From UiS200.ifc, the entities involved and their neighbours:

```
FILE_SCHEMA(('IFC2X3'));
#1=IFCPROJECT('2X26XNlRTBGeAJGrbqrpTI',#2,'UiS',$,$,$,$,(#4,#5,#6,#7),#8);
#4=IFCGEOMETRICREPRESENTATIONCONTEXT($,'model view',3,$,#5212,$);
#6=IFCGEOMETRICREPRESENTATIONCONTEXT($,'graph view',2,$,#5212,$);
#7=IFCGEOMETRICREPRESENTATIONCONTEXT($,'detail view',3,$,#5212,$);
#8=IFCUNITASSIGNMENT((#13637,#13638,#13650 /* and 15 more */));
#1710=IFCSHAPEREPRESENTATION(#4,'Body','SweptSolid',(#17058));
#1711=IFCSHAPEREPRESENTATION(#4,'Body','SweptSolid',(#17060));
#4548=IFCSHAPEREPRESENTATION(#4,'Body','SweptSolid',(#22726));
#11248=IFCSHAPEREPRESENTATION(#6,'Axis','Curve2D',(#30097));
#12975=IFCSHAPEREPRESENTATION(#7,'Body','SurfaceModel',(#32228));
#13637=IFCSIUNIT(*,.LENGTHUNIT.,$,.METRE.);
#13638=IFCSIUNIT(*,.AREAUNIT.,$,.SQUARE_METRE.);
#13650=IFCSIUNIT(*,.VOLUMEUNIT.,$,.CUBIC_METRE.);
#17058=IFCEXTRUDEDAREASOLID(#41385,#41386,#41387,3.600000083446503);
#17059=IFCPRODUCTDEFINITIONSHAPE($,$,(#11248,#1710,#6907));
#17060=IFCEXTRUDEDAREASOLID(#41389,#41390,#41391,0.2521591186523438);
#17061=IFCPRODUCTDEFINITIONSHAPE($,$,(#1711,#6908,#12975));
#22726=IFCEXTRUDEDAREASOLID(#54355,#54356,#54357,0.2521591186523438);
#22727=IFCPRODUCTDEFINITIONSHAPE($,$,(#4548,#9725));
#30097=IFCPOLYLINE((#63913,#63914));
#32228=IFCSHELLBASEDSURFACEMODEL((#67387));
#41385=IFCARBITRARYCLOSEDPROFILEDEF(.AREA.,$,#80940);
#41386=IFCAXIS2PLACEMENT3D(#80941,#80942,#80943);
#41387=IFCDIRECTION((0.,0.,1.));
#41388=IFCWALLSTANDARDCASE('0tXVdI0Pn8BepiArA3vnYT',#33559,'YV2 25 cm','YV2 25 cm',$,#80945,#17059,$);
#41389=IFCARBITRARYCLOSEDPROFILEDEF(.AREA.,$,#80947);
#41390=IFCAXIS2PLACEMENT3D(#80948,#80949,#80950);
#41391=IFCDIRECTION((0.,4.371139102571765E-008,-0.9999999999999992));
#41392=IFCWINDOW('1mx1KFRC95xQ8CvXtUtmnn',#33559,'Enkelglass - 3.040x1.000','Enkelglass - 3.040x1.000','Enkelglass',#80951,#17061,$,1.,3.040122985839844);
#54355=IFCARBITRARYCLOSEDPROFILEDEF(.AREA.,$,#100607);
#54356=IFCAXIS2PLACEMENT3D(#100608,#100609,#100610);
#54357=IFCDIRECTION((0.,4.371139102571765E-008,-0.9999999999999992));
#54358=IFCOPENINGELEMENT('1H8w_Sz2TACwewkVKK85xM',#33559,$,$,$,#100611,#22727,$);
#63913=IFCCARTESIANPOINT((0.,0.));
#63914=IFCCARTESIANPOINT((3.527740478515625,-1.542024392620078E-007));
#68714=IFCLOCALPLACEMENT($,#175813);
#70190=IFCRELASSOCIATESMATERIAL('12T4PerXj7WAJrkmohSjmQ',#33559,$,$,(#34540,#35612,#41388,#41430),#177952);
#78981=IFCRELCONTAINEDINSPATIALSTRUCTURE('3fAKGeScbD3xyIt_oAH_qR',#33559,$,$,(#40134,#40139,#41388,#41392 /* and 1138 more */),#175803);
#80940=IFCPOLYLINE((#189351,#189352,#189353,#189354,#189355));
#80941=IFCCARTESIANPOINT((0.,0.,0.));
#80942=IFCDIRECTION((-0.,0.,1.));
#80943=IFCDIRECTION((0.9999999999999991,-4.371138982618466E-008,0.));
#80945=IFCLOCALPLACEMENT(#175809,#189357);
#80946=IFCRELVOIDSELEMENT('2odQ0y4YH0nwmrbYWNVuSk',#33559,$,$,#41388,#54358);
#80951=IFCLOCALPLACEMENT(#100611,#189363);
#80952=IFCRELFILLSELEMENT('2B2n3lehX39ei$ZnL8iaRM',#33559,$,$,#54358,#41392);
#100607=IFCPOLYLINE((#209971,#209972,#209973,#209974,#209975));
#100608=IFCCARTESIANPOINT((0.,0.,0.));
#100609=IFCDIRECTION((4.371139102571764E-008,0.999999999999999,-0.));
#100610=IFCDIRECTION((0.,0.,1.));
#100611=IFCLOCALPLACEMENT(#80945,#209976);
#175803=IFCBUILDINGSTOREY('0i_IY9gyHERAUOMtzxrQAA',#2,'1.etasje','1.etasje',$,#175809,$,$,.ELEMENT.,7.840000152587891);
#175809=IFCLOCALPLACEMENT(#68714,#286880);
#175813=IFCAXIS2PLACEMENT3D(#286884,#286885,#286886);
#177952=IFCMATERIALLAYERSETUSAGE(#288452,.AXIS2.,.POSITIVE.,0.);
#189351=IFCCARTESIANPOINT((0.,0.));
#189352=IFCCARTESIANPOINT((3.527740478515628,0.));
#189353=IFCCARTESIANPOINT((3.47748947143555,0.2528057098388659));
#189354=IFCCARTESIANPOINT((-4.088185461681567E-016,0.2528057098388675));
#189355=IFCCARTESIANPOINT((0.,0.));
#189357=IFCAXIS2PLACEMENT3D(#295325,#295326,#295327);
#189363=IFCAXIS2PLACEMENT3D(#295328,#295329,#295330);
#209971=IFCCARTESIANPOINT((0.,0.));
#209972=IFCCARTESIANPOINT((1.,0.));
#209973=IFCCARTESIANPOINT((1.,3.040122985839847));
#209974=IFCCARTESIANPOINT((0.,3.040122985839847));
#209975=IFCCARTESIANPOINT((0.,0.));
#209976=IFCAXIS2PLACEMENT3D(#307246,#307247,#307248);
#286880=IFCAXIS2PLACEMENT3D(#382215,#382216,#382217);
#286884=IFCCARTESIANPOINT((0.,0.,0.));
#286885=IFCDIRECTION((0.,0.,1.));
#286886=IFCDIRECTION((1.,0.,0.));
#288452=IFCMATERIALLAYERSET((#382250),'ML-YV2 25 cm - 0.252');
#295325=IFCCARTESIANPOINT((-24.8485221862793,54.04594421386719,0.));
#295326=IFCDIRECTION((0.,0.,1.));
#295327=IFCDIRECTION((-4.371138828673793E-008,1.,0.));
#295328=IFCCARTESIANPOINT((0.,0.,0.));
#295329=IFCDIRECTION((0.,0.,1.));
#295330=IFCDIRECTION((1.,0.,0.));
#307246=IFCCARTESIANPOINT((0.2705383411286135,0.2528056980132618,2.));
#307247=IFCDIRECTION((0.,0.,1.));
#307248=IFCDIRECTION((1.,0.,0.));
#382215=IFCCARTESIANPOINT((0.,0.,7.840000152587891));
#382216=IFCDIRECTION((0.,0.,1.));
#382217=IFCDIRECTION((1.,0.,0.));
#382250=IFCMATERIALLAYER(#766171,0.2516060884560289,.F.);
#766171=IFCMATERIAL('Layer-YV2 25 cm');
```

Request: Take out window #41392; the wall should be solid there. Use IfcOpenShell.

```python
import ifcopenshell
import ifcopenshell.api.feature
import ifcopenshell.api.root
import ifcopenshell.geom
import ifcopenshell.util.shape

model = ifcopenshell.open("UiS200.ifc")
settings = ifcopenshell.geom.settings()


def volume(element):
    """Net volume in cubic metres, openings subtracted."""
    shape = ifcopenshell.geom.create_shape(settings, element)
    return ifcopenshell.util.shape.get_volume(shape.geometry)


window = model.by_guid("1mx1KFRC95xQ8CvXtUtmnn")
opening = window.FillsVoids[0].RelatingOpeningElement
wall = opening.VoidsElements[0].RelatingBuildingElement
before = volume(wall)

ifcopenshell.api.root.remove_product(model, product=window)
ifcopenshell.api.feature.remove_feature(model, feature=opening)

after = volume(wall)

print(f"wall volume {before:.3f} -> {after:.3f} m3")

model.write("UiS200_edited.ifc")
```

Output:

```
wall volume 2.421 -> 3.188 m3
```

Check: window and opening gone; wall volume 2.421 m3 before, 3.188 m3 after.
